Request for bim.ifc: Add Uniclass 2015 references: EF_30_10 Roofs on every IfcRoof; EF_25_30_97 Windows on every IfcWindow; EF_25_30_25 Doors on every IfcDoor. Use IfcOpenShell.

First a look at what the model holds.

```python
import ifcopenshell

model = ifcopenshell.open("bim.ifc")
print(model.schema)
print("classifications:", [c.Name for c in model.by_type("IfcClassification")])
for ifc_class in ("IfcDoor", "IfcRoof", "IfcStair", "IfcWall", "IfcWindow"):
    print(ifc_class, len(model.by_type(ifc_class)))
```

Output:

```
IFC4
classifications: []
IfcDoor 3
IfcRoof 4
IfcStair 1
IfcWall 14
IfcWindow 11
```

```python
import ifcopenshell
import ifcopenshell.api.classification

model = ifcopenshell.open("bim.ifc")

system = ifcopenshell.api.classification.add_classification(model, classification="Uniclass 2015")

codes = {
    "IfcRoof": ("EF_30_10", "Roofs"),
    "IfcWindow": ("EF_25_30_97", "Windows"),
    "IfcDoor": ("EF_25_30_25", "Doors"),
}
for ifc_class, (code, name) in codes.items():
    products = model.by_type(ifc_class)
    ifcopenshell.api.classification.add_reference(
        model, products=products, classification=system, identification=code, name=name
    )
    print(code, len(products))

model.write("bim_updated.ifc")
```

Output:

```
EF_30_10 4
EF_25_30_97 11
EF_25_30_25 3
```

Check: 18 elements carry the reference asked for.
